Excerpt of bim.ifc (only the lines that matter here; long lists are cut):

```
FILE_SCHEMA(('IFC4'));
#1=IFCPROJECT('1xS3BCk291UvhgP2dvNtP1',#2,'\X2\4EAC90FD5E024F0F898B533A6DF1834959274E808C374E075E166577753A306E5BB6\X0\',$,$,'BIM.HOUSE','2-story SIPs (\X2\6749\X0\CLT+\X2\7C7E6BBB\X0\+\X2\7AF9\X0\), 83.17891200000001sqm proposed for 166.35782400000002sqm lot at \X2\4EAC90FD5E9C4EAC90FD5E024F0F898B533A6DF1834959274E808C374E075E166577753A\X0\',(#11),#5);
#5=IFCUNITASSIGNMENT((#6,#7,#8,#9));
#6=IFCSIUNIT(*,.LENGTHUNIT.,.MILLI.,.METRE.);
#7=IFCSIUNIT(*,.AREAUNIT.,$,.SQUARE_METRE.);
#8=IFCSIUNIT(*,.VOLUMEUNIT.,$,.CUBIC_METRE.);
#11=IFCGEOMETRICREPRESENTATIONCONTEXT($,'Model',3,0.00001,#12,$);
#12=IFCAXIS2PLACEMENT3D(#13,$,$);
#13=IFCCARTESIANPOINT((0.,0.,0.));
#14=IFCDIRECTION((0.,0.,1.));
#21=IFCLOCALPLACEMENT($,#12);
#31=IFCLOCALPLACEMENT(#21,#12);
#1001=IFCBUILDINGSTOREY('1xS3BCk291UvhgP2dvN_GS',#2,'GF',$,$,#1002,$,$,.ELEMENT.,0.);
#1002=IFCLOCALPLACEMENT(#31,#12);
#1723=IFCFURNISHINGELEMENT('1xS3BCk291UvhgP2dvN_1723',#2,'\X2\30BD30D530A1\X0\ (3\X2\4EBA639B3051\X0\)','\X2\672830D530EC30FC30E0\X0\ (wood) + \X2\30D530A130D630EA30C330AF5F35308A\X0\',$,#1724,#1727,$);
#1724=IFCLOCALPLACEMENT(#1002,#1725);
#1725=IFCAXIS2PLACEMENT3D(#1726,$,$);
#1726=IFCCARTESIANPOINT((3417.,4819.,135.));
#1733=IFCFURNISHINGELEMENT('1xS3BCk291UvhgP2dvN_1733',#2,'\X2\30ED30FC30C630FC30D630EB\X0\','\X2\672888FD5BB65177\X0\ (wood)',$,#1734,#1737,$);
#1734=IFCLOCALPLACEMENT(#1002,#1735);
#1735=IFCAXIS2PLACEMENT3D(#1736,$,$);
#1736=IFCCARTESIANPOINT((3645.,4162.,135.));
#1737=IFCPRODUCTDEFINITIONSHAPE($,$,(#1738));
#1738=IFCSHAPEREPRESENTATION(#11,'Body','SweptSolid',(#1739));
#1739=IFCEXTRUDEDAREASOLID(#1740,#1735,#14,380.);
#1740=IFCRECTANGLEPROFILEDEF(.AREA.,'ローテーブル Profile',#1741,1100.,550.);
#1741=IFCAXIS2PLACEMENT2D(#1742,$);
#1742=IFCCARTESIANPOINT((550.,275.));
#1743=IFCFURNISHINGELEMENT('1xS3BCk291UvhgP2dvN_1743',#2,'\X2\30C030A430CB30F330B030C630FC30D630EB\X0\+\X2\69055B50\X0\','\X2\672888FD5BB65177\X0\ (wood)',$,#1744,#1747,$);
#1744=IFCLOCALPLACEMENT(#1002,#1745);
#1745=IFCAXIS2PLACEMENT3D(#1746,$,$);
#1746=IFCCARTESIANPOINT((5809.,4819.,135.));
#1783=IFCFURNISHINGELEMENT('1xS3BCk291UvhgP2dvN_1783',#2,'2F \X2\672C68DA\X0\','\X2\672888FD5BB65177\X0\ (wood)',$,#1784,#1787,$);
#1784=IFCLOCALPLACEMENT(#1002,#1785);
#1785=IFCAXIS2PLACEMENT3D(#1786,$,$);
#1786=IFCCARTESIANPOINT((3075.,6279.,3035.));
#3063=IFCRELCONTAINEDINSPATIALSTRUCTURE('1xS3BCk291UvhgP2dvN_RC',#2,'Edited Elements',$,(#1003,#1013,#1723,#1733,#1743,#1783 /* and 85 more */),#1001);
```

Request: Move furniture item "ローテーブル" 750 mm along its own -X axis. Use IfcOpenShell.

```python
import ifcopenshell
import ifcopenshell.api.geometry
import ifcopenshell.util.placement

model = ifcopenshell.open("bim.ifc")

item = model.by_guid("1xS3BCk291UvhgP2dvN_1733")
matrix = ifcopenshell.util.placement.get_local_placement(item.ObjectPlacement)
matrix[:3, 3] -= matrix[:3, 0] * 750.0
ifcopenshell.api.geometry.edit_object_placement(model, product=item, matrix=matrix, is_si=False)

print(ifcopenshell.util.placement.get_local_placement(item.ObjectPlacement).round(3) + 0.0)

model.write("bim_updated.ifc")
```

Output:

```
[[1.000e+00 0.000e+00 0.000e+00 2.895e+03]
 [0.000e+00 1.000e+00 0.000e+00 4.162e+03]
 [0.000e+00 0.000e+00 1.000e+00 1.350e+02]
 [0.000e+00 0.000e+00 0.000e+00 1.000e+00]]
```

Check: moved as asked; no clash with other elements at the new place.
